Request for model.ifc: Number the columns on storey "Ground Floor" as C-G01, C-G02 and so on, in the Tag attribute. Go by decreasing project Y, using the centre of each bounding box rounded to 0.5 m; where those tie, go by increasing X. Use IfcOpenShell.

First a look at what the model holds.

```python
import ifcopenshell
import ifcopenshell.util.element
import ifcopenshell.util.placement

model = ifcopenshell.open("model.ifc")
print(model.schema)
storey = next(s for s in model.by_type("IfcBuildingStorey") if s.Name == "Ground Floor")
columns = [e for e in ifcopenshell.util.element.get_decomposition(storey) if e.is_a("IfcColumn")]
for e in sorted(columns, key=lambda e: e.id()):
    origin = ifcopenshell.util.placement.get_local_placement(e.ObjectPlacement)[:3, 3]
    print(e.id(), e.Tag, e.Name, origin.round(2) + 0.0, sep=" | ")
```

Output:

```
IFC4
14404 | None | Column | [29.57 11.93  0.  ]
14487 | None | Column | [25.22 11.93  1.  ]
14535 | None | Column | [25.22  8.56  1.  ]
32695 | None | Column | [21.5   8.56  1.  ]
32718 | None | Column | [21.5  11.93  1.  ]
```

```python
import ifcopenshell
import ifcopenshell.geom
import ifcopenshell.util.element
import ifcopenshell.util.shape

model = ifcopenshell.open("model.ifc")
settings = ifcopenshell.geom.settings()
settings.set("use-world-coords", True)


def centre(element):
    shape = ifcopenshell.geom.create_shape(settings, element)
    return ifcopenshell.util.shape.get_bbox_centroid(shape.geometry)


storey = next(s for s in model.by_type("IfcBuildingStorey") if s.Name == "Ground Floor")
columns = [e for e in ifcopenshell.util.element.get_decomposition(storey) if e.is_a("IfcColumn")]

# Insertion points can sit at a corner or the storey origin, so sort by the geometry (in metres).
centres = {e: centre(e) for e in columns}
columns.sort(key=lambda e: (-round(centres[e][1] / 0.5), centres[e][0]))

for i, e in enumerate(columns, start=1):
    number = f"C-G{i:02d}"
    e.Tag = number
    print(e.id(), number)

model.write("model_updated.ifc")
```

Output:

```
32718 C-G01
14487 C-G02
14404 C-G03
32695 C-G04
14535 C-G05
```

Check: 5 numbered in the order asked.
